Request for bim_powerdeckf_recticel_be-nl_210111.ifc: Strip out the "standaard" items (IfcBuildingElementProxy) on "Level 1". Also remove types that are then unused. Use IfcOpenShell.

First a look at what the model holds.

```python
import ifcopenshell
import ifcopenshell.util.element

model = ifcopenshell.open("bim_powerdeckf_recticel_be-nl_210111.ifc")
print(model.schema)
storey = next(s for s in model.by_type("IfcBuildingStorey") if s.Name == "Level 1")
proxies = [e for e in ifcopenshell.util.element.get_decomposition(storey) if e.is_a("IfcBuildingElementProxy")]
seen = {}
for e in proxies:
    element_type = ifcopenshell.util.element.get_type(e)
    name = element_type.Name if element_type not in (None, e) else None
    seen[name] = seen.get(name, 0) + 1
for name, count in sorted(seen.items(), key=str):
    print(count, "x", name)
```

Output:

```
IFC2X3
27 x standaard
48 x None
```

```python
import ifcopenshell
import ifcopenshell.api.root
import ifcopenshell.util.element

model = ifcopenshell.open("bim_powerdeckf_recticel_be-nl_210111.ifc")

storey = next(s for s in model.by_type("IfcBuildingStorey") if s.Name == "Level 1")
proxies = [e for e in ifcopenshell.util.element.get_decomposition(storey) if e.is_a("IfcBuildingElementProxy")]
targets = [e for e in proxies if (t := ifcopenshell.util.element.get_type(e)) not in (None, e) and t.Name == "standaard"]
types = {ifcopenshell.util.element.get_type(e) for e in targets} - {None, *targets}

for e in targets:
    ifcopenshell.api.root.remove_product(model, product=e)
print(len(targets), "removed")

unused = [t for t in types if not ifcopenshell.util.element.get_types(t)]
for t in unused:
    ifcopenshell.api.root.remove_product(model, product=t)
print(len(unused), "unused types removed")

model.write("bim_powerdeckf_recticel_be-nl_210111_updated.ifc")
```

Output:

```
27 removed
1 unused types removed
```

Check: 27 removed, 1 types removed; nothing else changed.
